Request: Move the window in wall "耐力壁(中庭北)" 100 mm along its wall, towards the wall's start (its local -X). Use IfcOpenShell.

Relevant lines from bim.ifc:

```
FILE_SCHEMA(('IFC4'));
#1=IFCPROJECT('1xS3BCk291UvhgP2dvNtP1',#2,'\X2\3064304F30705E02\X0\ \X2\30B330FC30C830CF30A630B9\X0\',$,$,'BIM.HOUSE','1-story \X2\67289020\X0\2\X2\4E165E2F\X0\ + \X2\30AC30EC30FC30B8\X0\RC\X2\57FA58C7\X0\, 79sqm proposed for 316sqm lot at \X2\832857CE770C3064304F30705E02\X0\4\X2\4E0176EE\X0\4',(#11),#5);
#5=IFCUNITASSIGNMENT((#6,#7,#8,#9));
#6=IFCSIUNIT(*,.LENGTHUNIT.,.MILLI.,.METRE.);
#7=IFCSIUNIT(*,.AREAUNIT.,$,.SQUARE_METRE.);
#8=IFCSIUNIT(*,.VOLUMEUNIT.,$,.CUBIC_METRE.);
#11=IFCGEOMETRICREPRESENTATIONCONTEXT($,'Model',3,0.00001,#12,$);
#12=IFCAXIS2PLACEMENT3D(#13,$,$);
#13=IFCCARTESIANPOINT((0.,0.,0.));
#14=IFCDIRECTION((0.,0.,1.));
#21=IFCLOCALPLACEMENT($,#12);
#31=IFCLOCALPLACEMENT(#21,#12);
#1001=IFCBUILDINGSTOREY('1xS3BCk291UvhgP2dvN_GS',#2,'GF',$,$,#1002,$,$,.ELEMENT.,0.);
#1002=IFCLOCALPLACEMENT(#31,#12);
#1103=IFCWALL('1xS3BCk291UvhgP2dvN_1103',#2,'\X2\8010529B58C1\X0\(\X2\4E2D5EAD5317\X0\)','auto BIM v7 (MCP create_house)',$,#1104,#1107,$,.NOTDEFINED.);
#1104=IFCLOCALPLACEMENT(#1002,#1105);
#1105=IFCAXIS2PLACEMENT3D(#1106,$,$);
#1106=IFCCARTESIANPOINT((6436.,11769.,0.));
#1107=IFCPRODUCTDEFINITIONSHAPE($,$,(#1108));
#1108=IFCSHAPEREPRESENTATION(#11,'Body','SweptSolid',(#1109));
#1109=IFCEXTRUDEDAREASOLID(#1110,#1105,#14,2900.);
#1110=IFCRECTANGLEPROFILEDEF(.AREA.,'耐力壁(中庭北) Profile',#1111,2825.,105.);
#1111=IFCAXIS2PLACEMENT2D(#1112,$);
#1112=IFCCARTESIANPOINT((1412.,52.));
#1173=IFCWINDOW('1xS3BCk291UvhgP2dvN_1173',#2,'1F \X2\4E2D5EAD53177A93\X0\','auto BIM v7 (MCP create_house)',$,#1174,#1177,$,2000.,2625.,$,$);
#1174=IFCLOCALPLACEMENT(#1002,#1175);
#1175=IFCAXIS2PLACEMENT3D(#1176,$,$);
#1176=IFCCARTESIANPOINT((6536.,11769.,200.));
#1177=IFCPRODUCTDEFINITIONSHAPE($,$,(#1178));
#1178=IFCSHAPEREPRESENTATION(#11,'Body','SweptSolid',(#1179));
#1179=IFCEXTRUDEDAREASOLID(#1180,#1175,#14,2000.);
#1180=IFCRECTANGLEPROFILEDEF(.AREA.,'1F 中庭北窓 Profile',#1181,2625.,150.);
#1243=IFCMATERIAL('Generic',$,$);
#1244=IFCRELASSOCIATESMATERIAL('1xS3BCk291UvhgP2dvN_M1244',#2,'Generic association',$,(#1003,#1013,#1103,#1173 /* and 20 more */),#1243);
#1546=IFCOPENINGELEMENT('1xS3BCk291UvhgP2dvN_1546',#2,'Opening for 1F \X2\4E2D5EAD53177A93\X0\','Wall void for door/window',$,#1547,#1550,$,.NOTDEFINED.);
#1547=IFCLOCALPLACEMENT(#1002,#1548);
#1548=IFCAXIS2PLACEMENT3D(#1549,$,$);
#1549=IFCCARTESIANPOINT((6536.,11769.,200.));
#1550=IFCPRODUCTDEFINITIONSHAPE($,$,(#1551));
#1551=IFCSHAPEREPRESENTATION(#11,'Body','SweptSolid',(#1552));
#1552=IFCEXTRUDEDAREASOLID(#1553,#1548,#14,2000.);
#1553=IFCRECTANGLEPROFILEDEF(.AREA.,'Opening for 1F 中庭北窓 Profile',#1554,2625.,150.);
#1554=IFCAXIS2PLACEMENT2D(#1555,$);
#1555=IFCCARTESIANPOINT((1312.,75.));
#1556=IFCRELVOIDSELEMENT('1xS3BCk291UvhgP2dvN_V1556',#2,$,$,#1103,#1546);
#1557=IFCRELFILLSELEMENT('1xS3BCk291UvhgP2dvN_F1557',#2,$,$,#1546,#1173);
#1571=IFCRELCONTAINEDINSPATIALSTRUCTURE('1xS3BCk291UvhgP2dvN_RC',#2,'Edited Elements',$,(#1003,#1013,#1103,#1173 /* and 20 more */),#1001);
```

```python
import ifcopenshell
import ifcopenshell.api.geometry
import ifcopenshell.util.placement
import ifcopenshell.util.unit

model = ifcopenshell.open("bim.ifc")
unit_scale = ifcopenshell.util.unit.calculate_unit_scale(model)

window = model.by_guid("1xS3BCk291UvhgP2dvN_1173")
opening = window.FillsVoids[0].RelatingOpeningElement
wall = opening.VoidsElements[0].RelatingBuildingElement

wall_matrix = ifcopenshell.util.placement.get_local_placement(wall.ObjectPlacement)
shift = wall_matrix[:3, 0] * -0.1 / unit_scale
before = ifcopenshell.util.placement.get_local_placement(window.ObjectPlacement)[:3, 3].copy()

# The window is not placed relative to its opening, so move both.
for product in (opening, window):
    matrix = ifcopenshell.util.placement.get_local_placement(product.ObjectPlacement)
    matrix[:3, 3] += shift
    ifcopenshell.api.geometry.edit_object_placement(model, product=product, matrix=matrix, is_si=False)

after = ifcopenshell.util.placement.get_local_placement(window.ObjectPlacement)[:3, 3]
print("window moved by", (after - before).round(3) + 0.0)

model.write("bim_edited.ifc")
```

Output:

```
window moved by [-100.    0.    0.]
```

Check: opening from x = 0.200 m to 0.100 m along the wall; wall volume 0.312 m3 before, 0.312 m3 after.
